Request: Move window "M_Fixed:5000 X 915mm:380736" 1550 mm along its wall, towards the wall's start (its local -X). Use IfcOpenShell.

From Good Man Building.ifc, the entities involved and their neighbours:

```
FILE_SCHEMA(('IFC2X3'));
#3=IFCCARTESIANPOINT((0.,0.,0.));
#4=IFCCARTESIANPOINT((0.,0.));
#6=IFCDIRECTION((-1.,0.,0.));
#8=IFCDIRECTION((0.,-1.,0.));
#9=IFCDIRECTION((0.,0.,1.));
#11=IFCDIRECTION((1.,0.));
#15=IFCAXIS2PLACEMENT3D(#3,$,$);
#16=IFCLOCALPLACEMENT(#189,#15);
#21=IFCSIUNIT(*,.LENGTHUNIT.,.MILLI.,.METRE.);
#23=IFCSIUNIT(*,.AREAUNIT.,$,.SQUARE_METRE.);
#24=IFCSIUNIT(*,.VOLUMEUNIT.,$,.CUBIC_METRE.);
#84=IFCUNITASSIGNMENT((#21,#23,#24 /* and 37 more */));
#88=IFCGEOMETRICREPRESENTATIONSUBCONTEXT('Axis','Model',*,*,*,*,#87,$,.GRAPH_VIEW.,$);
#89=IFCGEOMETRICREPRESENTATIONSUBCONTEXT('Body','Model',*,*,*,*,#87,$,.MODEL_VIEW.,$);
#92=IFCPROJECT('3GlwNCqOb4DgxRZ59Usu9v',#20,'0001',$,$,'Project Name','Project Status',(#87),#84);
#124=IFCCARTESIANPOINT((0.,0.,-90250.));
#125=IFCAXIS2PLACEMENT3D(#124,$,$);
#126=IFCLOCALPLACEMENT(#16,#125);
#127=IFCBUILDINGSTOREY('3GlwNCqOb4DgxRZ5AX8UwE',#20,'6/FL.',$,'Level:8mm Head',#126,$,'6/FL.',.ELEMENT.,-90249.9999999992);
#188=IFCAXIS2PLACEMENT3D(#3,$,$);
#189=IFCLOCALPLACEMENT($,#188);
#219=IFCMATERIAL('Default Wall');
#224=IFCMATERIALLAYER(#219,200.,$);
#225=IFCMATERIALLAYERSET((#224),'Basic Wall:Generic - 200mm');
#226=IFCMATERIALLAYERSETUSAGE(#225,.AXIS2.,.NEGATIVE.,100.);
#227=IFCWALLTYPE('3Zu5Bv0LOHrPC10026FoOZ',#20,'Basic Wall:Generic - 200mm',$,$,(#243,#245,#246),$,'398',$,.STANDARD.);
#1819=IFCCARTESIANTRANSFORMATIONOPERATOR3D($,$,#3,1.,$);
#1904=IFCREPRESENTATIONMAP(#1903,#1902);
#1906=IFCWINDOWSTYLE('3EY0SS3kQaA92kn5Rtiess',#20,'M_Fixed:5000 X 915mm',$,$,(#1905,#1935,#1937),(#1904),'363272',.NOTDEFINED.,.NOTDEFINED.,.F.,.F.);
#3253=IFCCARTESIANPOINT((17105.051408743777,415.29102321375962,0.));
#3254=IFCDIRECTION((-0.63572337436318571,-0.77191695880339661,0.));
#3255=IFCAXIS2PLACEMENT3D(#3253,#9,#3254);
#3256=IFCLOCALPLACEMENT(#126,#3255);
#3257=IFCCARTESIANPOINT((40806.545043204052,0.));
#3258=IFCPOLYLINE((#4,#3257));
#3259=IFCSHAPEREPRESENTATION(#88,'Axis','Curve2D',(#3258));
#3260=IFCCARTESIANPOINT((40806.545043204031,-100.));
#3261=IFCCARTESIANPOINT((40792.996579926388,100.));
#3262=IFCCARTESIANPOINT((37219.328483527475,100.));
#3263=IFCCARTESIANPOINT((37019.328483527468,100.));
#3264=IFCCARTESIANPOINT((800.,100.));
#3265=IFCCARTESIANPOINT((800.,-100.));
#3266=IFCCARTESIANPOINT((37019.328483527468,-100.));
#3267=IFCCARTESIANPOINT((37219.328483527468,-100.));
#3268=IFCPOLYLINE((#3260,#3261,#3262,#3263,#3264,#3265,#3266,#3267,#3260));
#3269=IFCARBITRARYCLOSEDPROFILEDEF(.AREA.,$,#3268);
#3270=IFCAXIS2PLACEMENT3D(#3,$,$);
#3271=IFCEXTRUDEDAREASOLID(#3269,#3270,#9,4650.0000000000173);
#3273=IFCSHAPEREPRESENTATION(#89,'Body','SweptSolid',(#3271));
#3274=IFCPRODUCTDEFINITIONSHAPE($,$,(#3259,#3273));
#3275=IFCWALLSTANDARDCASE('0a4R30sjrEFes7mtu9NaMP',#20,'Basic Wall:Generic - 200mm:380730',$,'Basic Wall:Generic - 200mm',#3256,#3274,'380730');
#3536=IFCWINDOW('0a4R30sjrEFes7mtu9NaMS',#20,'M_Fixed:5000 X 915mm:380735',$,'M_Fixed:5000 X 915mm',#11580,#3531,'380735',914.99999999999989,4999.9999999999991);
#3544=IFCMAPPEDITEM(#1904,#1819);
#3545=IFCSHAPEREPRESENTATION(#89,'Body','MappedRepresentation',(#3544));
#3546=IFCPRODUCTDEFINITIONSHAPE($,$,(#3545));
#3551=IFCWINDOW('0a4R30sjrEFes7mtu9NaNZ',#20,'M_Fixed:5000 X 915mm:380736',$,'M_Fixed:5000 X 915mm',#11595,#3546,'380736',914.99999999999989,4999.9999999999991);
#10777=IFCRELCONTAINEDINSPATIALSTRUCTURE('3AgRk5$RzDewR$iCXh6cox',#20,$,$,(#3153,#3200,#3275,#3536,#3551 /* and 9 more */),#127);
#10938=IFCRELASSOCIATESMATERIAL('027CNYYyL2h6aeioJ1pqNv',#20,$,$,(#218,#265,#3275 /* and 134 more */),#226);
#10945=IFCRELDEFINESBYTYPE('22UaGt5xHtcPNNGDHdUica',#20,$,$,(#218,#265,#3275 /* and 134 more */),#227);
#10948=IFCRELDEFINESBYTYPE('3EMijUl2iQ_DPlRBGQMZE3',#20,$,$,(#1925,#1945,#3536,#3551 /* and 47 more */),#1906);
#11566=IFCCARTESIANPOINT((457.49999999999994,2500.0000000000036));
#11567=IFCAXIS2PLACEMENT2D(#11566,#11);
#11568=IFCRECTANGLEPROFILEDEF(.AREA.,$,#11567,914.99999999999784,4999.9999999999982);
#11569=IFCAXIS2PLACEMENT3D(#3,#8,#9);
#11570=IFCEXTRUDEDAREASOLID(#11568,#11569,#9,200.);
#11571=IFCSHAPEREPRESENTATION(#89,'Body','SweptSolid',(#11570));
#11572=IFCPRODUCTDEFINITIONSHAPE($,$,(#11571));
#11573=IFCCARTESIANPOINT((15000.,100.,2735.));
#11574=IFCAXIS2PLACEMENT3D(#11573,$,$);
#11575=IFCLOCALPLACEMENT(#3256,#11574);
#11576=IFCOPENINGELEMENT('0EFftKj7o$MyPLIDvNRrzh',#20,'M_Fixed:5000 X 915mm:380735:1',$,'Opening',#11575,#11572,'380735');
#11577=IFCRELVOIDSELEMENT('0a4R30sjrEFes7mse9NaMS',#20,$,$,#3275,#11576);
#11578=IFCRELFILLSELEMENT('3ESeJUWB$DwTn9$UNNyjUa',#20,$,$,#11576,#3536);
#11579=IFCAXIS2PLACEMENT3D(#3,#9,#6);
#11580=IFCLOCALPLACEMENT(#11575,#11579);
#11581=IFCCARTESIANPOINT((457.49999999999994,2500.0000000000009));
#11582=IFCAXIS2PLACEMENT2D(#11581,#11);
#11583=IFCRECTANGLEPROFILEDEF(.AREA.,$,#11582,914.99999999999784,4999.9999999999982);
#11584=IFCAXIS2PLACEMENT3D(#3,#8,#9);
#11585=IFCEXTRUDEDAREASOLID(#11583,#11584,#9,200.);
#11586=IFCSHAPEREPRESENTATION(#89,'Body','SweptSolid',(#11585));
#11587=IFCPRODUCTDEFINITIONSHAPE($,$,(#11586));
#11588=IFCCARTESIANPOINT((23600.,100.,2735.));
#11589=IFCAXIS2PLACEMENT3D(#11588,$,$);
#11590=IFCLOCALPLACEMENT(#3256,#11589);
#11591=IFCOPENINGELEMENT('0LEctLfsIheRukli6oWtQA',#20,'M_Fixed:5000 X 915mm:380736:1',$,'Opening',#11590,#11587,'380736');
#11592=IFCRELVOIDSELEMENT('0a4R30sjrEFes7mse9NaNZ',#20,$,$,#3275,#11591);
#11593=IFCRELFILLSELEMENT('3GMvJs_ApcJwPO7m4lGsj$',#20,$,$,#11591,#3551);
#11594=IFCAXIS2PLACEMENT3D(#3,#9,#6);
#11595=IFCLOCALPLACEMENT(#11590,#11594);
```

```python
import ifcopenshell
import ifcopenshell.api.geometry
import ifcopenshell.util.placement

model = ifcopenshell.open("Good Man Building.ifc")

window = model.by_guid("0a4R30sjrEFes7mtu9NaNZ")
opening = window.FillsVoids[0].RelatingOpeningElement
wall = opening.VoidsElements[0].RelatingBuildingElement

wall_matrix = ifcopenshell.util.placement.get_local_placement(wall.ObjectPlacement)
shift = wall_matrix[:3, 0] * -1550.0
before = ifcopenshell.util.placement.get_local_placement(window.ObjectPlacement)[:3, 3].copy()

# The window is placed relative to its opening, so it follows when the opening moves.
matrix = ifcopenshell.util.placement.get_local_placement(opening.ObjectPlacement)
matrix[:3, 3] += shift
ifcopenshell.api.geometry.edit_object_placement(
    model, product=opening, matrix=matrix, is_si=False, should_transform_children=True
)

after = ifcopenshell.util.placement.get_local_placement(window.ObjectPlacement)[:3, 3]
print("window moved by", (after - before).round(3) + 0.0)

model.write("Good Man Building-out.ifc")
```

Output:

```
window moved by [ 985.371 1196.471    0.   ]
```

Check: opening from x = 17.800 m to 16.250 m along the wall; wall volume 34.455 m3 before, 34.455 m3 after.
